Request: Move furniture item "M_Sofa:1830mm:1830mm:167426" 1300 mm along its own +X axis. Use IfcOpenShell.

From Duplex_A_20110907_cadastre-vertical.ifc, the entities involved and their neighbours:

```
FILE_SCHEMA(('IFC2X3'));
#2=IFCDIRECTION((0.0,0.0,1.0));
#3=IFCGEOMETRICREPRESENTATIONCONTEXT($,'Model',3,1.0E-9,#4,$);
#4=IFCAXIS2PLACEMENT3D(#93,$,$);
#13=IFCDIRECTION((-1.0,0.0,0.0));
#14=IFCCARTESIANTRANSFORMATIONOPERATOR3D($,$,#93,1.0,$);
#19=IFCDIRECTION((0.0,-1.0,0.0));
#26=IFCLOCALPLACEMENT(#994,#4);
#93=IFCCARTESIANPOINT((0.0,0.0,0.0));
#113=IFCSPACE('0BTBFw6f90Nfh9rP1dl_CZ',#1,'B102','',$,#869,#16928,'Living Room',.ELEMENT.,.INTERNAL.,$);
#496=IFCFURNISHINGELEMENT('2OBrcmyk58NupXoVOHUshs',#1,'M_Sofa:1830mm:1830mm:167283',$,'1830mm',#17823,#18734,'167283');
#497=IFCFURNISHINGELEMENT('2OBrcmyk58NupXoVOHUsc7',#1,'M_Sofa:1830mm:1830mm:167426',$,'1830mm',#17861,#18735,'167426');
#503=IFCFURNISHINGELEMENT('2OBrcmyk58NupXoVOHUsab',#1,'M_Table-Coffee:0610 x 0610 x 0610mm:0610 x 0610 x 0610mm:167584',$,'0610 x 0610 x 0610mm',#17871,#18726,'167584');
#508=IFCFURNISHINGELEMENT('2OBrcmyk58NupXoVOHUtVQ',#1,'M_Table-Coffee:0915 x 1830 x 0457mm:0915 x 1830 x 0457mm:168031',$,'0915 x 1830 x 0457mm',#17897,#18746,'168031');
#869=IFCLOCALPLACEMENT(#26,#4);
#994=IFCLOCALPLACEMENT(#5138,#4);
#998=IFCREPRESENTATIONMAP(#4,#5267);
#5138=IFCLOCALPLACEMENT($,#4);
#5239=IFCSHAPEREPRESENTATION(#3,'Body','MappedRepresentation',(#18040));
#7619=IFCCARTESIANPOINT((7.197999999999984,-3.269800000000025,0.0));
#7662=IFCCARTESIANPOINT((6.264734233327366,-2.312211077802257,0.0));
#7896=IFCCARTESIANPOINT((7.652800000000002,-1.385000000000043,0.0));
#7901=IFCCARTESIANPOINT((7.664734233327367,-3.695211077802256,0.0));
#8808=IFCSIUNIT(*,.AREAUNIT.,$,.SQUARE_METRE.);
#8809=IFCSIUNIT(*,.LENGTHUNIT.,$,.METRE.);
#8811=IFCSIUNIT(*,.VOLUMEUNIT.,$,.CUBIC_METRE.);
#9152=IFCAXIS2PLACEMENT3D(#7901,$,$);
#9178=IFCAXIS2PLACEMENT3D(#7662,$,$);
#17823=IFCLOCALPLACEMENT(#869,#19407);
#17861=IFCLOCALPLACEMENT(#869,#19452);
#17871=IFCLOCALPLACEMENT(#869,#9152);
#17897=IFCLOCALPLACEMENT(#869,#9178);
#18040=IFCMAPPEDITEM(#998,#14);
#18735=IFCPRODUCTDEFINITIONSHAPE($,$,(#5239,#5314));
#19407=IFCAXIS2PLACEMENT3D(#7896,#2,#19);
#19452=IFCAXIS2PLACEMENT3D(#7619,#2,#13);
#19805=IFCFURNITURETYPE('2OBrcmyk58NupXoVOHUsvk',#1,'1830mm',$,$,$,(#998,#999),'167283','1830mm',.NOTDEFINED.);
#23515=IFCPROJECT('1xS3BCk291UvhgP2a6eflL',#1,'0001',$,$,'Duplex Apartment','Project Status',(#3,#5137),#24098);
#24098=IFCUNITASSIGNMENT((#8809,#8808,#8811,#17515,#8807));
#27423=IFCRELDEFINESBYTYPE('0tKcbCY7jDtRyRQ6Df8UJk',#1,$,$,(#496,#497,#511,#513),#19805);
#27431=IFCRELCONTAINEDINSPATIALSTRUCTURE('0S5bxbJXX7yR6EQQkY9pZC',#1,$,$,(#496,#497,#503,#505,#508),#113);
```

```python
import ifcopenshell
import ifcopenshell.api.geometry
import ifcopenshell.util.placement
import ifcopenshell.util.unit

model = ifcopenshell.open("Duplex_A_20110907_cadastre-vertical.ifc")
unit_scale = ifcopenshell.util.unit.calculate_unit_scale(model)

item = model.by_guid("2OBrcmyk58NupXoVOHUsc7")
matrix = ifcopenshell.util.placement.get_local_placement(item.ObjectPlacement)
matrix[:3, 3] += matrix[:3, 0] * 1.3 / unit_scale
ifcopenshell.api.geometry.edit_object_placement(model, product=item, matrix=matrix, is_si=False)

print(ifcopenshell.util.placement.get_local_placement(item.ObjectPlacement).round(3) + 0.0)

model.write("Duplex_A_20110907_cadastre-vertical_v2.ifc")
```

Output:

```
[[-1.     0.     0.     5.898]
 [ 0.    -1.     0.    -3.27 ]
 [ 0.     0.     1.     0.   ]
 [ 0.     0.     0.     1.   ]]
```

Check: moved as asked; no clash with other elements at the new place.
